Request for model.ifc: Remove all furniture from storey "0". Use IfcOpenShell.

First a look at what the model holds.

```python
import ifcopenshell
import ifcopenshell.util.element

model = ifcopenshell.open("model.ifc")
print(model.schema)
storey = next(s for s in model.by_type("IfcBuildingStorey") if s.Name == "0")
furniture = [e for e in ifcopenshell.util.element.get_decomposition(storey) if e.is_a("IfcFurnishingElement")]
seen = {}
for e in furniture:
    element_type = ifcopenshell.util.element.get_type(e)
    name = element_type.Name if element_type not in (None, e) else None
    seen[name] = seen.get(name, 0) + 1
for name, count in sorted(seen.items(), key=str):
    print(count, "x", name)
```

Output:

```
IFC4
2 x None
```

```python
import ifcopenshell
import ifcopenshell.api.root
import ifcopenshell.util.element

model = ifcopenshell.open("model.ifc")

storey = next(s for s in model.by_type("IfcBuildingStorey") if s.Name == "0")
furniture = [e for e in ifcopenshell.util.element.get_decomposition(storey) if e.is_a("IfcFurnishingElement")]

for e in furniture:
    ifcopenshell.api.root.remove_product(model, product=e)
print(len(furniture), "removed")

model.write("model_rev.ifc")
```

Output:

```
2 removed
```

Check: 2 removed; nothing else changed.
